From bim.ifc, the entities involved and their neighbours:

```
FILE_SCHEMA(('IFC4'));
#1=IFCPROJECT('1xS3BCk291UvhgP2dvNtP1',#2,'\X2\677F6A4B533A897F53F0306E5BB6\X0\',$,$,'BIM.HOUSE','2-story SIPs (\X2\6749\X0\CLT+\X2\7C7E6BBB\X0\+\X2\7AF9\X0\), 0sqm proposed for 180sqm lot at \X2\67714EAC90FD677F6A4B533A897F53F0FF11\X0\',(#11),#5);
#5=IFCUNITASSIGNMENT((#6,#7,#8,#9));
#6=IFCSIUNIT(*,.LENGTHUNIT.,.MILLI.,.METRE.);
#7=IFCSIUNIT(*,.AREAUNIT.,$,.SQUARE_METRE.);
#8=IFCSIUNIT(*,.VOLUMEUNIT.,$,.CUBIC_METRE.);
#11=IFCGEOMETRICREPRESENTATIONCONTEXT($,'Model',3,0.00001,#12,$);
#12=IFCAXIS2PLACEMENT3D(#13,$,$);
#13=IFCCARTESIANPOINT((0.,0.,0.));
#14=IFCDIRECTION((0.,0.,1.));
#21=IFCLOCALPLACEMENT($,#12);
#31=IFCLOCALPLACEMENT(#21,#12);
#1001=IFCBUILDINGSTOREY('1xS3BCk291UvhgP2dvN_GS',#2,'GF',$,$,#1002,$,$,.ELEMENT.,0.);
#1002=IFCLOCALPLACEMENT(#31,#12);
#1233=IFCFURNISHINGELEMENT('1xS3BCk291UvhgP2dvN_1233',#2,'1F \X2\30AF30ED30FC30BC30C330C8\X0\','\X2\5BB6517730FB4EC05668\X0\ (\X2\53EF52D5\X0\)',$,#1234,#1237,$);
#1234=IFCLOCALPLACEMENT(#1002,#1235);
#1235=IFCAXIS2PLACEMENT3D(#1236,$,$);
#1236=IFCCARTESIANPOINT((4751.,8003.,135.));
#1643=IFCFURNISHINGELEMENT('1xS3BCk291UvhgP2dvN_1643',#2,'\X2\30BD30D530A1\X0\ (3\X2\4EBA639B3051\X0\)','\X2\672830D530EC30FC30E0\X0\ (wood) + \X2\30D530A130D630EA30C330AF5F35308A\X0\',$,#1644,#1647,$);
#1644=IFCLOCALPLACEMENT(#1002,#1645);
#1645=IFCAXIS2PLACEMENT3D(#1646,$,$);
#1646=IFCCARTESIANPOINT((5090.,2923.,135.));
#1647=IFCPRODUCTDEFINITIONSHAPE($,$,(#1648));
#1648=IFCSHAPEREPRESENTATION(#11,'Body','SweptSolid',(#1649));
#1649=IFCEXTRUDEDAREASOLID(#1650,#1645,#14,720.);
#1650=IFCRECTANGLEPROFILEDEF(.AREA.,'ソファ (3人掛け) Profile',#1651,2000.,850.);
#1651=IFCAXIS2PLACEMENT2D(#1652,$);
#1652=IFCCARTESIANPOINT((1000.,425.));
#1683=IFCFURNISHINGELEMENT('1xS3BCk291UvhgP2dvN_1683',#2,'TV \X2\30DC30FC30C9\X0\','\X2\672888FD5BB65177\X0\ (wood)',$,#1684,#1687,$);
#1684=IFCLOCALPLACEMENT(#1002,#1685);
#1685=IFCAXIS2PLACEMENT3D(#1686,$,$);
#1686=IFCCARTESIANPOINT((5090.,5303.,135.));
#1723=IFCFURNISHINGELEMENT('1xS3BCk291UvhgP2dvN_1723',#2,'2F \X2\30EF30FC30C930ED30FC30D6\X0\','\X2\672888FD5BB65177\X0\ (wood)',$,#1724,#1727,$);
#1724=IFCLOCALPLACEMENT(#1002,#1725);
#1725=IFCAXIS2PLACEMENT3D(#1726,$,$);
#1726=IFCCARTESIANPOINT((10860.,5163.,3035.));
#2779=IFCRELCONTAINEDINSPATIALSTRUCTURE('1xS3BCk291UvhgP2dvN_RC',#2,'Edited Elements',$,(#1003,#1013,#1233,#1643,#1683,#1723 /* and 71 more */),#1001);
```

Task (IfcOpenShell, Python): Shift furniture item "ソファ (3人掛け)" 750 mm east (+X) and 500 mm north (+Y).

```python
import ifcopenshell
import ifcopenshell.api.geometry
import ifcopenshell.util.placement
import ifcopenshell.util.unit

model = ifcopenshell.open("bim.ifc")
unit_scale = ifcopenshell.util.unit.calculate_unit_scale(model)

item = model.by_guid("1xS3BCk291UvhgP2dvN_1643")
matrix = ifcopenshell.util.placement.get_local_placement(item.ObjectPlacement)
matrix[0, 3] += 0.75 / unit_scale
matrix[1, 3] += 0.5 / unit_scale
ifcopenshell.api.geometry.edit_object_placement(model, product=item, matrix=matrix, is_si=False)

print(ifcopenshell.util.placement.get_local_placement(item.ObjectPlacement).round(3) + 0.0)

model.write("bim_v2.ifc")
```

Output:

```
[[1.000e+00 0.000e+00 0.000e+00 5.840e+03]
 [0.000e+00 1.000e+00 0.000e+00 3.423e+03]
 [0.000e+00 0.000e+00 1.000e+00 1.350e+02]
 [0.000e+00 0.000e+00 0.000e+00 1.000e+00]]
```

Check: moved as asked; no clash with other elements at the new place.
